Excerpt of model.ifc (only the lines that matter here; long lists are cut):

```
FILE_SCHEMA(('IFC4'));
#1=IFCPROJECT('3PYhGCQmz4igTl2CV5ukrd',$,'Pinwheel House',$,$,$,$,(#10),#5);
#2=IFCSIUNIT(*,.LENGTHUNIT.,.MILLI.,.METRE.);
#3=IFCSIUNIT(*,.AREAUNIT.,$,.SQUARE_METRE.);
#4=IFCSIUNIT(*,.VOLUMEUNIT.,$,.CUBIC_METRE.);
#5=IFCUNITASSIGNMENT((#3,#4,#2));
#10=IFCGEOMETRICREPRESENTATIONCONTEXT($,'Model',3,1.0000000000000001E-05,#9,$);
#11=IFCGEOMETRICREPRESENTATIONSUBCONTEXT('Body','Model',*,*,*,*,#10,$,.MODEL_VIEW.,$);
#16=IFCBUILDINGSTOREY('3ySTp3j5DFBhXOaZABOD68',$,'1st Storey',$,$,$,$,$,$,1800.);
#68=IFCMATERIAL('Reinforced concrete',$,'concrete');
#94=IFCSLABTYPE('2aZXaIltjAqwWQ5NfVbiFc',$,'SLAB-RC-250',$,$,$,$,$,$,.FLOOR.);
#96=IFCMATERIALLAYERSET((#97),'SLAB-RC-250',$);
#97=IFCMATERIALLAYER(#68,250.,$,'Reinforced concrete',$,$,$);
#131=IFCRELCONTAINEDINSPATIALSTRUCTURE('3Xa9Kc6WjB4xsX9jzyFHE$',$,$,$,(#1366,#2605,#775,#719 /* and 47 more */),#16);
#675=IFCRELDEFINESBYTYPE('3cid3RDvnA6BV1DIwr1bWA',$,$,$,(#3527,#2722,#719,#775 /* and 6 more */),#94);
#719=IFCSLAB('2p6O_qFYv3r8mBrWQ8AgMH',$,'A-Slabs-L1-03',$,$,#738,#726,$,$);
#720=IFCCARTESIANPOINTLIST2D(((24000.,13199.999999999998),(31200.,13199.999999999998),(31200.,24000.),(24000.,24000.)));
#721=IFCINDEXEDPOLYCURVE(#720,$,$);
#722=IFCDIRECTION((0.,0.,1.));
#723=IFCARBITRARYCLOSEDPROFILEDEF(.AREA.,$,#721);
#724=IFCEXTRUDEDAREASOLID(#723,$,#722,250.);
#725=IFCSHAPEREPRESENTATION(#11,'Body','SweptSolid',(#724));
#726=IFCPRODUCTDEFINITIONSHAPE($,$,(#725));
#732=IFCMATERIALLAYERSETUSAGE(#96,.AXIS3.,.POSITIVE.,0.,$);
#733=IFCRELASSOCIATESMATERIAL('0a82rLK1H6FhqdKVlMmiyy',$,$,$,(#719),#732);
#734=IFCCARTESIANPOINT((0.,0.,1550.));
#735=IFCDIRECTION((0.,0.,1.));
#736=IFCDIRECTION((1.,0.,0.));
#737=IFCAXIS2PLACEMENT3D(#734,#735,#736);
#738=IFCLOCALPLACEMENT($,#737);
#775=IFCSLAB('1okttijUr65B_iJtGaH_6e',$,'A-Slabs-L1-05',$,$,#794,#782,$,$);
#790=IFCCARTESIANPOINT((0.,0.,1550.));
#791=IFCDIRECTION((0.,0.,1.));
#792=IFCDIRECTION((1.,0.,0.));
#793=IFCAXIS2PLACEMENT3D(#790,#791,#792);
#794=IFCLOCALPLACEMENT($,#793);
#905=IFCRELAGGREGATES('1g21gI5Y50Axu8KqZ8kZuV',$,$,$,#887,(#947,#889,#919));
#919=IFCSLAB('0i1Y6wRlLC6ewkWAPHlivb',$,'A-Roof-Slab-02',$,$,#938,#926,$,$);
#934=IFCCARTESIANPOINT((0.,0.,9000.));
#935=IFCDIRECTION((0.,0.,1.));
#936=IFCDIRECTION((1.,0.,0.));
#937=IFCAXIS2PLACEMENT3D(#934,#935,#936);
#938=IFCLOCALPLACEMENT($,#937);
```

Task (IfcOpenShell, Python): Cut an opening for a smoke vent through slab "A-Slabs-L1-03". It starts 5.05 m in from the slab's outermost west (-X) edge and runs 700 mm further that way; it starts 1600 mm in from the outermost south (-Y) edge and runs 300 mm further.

```python
import numpy as np
import ifcopenshell
import ifcopenshell.api.feature
import ifcopenshell.api.geometry
import ifcopenshell.api.root
import ifcopenshell.geom
import ifcopenshell.util.placement
import ifcopenshell.util.representation
import ifcopenshell.util.shape
import ifcopenshell.util.unit

model = ifcopenshell.open("model.ifc")
unit_scale = ifcopenshell.util.unit.calculate_unit_scale(model)
settings = ifcopenshell.geom.settings()


def volume(element):
    """Net volume in cubic metres, openings subtracted."""
    shape = ifcopenshell.geom.create_shape(settings, element)
    return ifcopenshell.util.shape.get_volume(shape.geometry)


slab = model.by_guid("2p6O_qFYv3r8mBrWQ8AgMH")
before = volume(slab)

# Extent in the slab's own axes, in metres. The edges named are its -X and -Y sides.
slab_shape = ifcopenshell.geom.create_shape(settings, slab)
vertices = ifcopenshell.util.shape.get_vertices(slab_shape.geometry)
x_min, y_min, bottom = vertices.min(axis=0)
top = vertices[:, 2].max()

opening = ifcopenshell.api.root.create_entity(model, ifc_class="IfcOpeningElement", name="Smoke vent opening", predefined_type="OPENING")
context = ifcopenshell.util.representation.get_context(model, "Model", "Body", "MODEL_VIEW")
width, depth = 0.7, 0.3
outline = [(0.0, 0.0), (width, 0.0), (width, depth), (0.0, depth), (0.0, 0.0)]
# Overshoot both faces by 50 mm so the cut is clean.
shape = ifcopenshell.api.geometry.add_slab_representation(
    model, context=context, depth=top - bottom + 0.1, polyline=outline
)
ifcopenshell.api.geometry.assign_representation(model, product=opening, representation=shape)

matrix = ifcopenshell.util.placement.get_local_placement(slab.ObjectPlacement)
matrix[:, 3] = matrix @ np.append(np.array([x_min + 5.05, y_min + 1.6, bottom - 0.05]) / unit_scale, 1.0)
ifcopenshell.api.geometry.edit_object_placement(model, product=opening, matrix=matrix, is_si=False)
ifcopenshell.api.feature.add_feature(model, feature=opening, element=slab)

after = volume(slab)

print(f"slab volume {before:.3f} -> {after:.3f} m3")

model.write("model_rev.ifc")
```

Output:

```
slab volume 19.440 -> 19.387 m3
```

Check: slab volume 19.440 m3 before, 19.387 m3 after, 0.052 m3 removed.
